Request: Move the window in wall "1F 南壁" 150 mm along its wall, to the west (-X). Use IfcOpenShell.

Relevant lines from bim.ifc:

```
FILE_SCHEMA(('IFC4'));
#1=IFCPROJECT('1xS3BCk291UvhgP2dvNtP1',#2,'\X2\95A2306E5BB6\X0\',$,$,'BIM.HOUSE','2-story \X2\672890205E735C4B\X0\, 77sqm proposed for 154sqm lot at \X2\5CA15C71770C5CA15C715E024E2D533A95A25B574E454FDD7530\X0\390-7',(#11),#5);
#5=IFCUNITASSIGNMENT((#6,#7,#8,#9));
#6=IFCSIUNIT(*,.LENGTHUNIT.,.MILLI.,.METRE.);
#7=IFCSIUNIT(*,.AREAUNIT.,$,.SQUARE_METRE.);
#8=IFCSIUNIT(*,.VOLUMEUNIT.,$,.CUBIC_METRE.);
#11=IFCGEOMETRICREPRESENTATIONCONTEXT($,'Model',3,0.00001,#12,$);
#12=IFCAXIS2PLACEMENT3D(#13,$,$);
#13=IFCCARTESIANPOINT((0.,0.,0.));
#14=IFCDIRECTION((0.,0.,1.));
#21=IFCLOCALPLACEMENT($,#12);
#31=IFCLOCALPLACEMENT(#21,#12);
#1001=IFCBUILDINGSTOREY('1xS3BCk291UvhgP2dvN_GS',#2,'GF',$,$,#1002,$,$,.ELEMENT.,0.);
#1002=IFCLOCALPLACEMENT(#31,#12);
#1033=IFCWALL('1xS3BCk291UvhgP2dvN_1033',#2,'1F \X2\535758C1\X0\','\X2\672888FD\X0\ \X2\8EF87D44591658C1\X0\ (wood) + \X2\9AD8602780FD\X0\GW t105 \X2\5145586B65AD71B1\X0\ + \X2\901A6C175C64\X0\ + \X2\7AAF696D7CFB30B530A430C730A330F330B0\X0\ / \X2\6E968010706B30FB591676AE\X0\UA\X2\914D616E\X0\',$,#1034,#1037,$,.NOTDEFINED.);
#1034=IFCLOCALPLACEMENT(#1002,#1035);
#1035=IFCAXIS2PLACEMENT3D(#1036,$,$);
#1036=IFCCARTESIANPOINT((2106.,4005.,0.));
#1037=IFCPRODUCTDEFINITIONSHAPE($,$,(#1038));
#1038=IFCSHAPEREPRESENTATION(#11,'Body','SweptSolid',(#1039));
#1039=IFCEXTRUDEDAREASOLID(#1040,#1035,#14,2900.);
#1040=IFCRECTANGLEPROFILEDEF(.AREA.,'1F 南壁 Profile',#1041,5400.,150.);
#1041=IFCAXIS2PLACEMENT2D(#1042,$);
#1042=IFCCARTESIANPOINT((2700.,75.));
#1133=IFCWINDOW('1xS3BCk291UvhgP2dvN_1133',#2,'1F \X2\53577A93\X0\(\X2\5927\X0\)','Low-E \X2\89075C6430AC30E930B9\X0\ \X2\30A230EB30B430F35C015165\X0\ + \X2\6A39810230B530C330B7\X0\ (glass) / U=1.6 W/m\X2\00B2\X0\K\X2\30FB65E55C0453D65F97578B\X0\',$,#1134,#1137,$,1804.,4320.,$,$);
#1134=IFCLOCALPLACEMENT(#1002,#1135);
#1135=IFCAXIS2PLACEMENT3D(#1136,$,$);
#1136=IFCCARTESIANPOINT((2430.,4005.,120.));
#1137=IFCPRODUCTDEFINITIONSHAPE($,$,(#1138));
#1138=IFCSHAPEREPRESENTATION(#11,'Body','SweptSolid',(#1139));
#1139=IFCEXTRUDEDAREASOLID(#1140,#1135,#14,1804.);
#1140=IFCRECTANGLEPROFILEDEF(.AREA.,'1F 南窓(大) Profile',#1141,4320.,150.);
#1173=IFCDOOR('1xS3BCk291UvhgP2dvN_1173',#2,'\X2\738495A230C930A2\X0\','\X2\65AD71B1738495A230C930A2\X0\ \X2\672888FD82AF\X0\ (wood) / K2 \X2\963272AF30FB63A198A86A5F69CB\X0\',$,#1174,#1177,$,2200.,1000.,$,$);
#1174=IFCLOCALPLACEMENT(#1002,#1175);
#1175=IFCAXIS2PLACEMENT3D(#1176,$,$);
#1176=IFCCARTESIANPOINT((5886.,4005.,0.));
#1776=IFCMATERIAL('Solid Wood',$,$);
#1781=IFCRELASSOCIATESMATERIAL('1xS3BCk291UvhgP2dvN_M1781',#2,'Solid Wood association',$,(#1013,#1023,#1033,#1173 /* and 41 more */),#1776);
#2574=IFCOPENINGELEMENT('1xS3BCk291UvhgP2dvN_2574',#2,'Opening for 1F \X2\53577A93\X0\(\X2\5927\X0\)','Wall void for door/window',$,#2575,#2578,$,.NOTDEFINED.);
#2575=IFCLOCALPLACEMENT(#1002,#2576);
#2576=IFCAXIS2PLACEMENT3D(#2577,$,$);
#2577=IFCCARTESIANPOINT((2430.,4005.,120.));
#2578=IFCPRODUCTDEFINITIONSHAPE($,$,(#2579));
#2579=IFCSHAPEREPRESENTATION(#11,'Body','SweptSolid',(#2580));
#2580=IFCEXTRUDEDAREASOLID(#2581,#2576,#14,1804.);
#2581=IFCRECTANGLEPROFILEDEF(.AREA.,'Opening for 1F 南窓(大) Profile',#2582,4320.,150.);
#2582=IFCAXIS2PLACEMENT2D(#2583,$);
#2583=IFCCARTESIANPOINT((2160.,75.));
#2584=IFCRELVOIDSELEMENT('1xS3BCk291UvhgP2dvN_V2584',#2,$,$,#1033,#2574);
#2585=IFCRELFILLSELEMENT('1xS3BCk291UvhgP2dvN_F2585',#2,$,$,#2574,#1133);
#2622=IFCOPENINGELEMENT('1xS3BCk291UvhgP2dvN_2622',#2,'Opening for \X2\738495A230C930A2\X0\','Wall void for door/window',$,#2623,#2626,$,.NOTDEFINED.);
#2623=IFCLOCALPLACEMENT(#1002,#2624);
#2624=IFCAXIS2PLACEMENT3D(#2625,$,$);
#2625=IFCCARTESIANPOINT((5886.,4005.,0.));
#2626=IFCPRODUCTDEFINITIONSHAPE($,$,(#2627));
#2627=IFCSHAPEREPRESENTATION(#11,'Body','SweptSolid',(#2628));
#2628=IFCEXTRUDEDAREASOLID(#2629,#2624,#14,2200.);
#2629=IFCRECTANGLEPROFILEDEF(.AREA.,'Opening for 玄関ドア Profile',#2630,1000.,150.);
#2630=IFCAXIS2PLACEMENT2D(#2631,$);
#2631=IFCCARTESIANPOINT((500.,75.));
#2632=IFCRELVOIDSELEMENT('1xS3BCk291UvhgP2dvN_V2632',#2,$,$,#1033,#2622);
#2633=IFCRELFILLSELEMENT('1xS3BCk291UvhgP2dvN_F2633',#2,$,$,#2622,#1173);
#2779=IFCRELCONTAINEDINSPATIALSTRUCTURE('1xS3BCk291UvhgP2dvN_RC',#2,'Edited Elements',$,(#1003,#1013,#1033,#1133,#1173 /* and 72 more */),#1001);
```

```python
import ifcopenshell
import ifcopenshell.api.geometry
import ifcopenshell.util.placement
import ifcopenshell.util.unit

model = ifcopenshell.open("bim.ifc")
unit_scale = ifcopenshell.util.unit.calculate_unit_scale(model)

window = model.by_guid("1xS3BCk291UvhgP2dvN_1133")
opening = window.FillsVoids[0].RelatingOpeningElement
wall = opening.VoidsElements[0].RelatingBuildingElement

wall_matrix = ifcopenshell.util.placement.get_local_placement(wall.ObjectPlacement)
shift = wall_matrix[:3, 0] * -0.15 / unit_scale
before = ifcopenshell.util.placement.get_local_placement(window.ObjectPlacement)[:3, 3].copy()

# The window is not placed relative to its opening, so move both.
for product in (opening, window):
    matrix = ifcopenshell.util.placement.get_local_placement(product.ObjectPlacement)
    matrix[:3, 3] += shift
    ifcopenshell.api.geometry.edit_object_placement(model, product=product, matrix=matrix, is_si=False)

after = ifcopenshell.util.placement.get_local_placement(window.ObjectPlacement)[:3, 3]
print("window moved by", (after - before).round(3) + 0.0)

model.write("bim_updated.ifc")
```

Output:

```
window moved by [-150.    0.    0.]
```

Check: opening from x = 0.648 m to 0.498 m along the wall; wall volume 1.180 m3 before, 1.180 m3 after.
